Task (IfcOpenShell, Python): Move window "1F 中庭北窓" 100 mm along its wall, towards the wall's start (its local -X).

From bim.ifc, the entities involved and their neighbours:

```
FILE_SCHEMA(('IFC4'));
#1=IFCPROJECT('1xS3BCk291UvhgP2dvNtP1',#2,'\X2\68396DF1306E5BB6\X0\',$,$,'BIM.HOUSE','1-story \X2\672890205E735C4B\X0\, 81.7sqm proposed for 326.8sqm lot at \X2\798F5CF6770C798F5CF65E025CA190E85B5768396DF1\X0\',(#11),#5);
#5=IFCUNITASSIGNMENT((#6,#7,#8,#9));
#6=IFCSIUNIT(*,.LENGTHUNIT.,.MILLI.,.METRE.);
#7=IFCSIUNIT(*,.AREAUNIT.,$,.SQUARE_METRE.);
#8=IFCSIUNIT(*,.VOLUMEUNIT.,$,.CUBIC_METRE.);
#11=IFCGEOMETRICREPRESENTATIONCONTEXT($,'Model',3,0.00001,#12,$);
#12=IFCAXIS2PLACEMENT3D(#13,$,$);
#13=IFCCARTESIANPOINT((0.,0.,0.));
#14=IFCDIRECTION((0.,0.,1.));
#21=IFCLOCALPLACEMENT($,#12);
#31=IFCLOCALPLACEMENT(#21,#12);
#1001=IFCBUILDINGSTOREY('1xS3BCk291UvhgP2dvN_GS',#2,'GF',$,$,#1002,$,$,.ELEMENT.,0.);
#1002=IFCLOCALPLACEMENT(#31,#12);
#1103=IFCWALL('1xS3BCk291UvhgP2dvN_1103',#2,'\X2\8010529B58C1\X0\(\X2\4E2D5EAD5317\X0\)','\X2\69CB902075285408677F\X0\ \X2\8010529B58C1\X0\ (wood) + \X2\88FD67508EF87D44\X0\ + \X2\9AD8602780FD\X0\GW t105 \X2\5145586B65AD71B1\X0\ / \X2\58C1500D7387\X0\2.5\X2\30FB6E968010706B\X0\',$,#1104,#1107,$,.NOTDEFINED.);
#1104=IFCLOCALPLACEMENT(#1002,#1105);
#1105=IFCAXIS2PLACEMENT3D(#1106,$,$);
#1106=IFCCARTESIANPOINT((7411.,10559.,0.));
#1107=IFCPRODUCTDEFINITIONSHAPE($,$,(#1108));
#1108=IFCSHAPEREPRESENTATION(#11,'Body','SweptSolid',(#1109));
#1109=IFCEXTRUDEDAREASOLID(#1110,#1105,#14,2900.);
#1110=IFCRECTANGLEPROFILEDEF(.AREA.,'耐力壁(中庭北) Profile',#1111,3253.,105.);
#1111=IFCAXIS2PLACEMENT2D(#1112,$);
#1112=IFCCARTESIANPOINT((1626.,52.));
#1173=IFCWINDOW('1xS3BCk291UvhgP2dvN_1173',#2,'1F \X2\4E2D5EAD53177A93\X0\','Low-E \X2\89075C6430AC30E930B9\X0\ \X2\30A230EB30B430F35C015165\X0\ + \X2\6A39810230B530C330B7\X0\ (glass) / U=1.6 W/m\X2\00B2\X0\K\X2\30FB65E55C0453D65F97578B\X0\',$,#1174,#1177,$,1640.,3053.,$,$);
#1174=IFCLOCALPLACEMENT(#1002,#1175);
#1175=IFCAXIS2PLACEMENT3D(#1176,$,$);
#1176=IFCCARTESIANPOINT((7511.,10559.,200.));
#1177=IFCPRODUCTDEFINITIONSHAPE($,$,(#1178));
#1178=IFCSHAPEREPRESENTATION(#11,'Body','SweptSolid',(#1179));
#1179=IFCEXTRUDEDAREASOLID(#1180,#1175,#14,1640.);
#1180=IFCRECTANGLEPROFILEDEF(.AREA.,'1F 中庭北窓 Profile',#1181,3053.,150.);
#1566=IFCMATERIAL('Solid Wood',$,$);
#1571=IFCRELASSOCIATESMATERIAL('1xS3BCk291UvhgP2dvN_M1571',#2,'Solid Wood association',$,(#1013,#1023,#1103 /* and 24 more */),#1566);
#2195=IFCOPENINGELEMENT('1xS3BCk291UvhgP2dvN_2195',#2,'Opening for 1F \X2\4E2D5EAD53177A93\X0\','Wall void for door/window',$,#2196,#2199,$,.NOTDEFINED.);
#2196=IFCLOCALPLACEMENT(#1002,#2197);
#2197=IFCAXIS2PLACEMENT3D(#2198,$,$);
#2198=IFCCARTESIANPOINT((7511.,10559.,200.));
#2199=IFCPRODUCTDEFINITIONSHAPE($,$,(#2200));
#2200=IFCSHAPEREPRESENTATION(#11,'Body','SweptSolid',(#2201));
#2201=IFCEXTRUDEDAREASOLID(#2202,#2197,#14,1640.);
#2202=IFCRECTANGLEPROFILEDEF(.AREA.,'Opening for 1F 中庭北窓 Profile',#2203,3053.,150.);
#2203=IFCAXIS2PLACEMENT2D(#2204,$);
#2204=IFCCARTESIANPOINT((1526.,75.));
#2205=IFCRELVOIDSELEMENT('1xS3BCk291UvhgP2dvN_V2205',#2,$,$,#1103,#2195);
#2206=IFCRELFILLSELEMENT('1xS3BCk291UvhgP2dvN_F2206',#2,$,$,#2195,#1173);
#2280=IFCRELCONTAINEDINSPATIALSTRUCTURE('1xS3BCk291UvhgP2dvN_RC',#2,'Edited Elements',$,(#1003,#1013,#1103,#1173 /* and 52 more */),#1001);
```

```python
import ifcopenshell
import ifcopenshell.api.geometry
import ifcopenshell.util.placement
import ifcopenshell.util.unit

model = ifcopenshell.open("bim.ifc")
unit_scale = ifcopenshell.util.unit.calculate_unit_scale(model)

window = model.by_guid("1xS3BCk291UvhgP2dvN_1173")
opening = window.FillsVoids[0].RelatingOpeningElement
wall = opening.VoidsElements[0].RelatingBuildingElement

wall_matrix = ifcopenshell.util.placement.get_local_placement(wall.ObjectPlacement)
shift = wall_matrix[:3, 0] * -0.1 / unit_scale
before = ifcopenshell.util.placement.get_local_placement(window.ObjectPlacement)[:3, 3].copy()

# The window is not placed relative to its opening, so move both.
for product in (opening, window):
    matrix = ifcopenshell.util.placement.get_local_placement(product.ObjectPlacement)
    matrix[:3, 3] += shift
    ifcopenshell.api.geometry.edit_object_placement(model, product=product, matrix=matrix, is_si=False)

after = ifcopenshell.util.placement.get_local_placement(window.ObjectPlacement)[:3, 3]
print("window moved by", (after - before).round(3) + 0.0)

model.write("bim_v2.ifc")
```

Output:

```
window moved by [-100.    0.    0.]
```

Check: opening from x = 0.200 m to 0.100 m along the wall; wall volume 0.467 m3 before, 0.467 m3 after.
